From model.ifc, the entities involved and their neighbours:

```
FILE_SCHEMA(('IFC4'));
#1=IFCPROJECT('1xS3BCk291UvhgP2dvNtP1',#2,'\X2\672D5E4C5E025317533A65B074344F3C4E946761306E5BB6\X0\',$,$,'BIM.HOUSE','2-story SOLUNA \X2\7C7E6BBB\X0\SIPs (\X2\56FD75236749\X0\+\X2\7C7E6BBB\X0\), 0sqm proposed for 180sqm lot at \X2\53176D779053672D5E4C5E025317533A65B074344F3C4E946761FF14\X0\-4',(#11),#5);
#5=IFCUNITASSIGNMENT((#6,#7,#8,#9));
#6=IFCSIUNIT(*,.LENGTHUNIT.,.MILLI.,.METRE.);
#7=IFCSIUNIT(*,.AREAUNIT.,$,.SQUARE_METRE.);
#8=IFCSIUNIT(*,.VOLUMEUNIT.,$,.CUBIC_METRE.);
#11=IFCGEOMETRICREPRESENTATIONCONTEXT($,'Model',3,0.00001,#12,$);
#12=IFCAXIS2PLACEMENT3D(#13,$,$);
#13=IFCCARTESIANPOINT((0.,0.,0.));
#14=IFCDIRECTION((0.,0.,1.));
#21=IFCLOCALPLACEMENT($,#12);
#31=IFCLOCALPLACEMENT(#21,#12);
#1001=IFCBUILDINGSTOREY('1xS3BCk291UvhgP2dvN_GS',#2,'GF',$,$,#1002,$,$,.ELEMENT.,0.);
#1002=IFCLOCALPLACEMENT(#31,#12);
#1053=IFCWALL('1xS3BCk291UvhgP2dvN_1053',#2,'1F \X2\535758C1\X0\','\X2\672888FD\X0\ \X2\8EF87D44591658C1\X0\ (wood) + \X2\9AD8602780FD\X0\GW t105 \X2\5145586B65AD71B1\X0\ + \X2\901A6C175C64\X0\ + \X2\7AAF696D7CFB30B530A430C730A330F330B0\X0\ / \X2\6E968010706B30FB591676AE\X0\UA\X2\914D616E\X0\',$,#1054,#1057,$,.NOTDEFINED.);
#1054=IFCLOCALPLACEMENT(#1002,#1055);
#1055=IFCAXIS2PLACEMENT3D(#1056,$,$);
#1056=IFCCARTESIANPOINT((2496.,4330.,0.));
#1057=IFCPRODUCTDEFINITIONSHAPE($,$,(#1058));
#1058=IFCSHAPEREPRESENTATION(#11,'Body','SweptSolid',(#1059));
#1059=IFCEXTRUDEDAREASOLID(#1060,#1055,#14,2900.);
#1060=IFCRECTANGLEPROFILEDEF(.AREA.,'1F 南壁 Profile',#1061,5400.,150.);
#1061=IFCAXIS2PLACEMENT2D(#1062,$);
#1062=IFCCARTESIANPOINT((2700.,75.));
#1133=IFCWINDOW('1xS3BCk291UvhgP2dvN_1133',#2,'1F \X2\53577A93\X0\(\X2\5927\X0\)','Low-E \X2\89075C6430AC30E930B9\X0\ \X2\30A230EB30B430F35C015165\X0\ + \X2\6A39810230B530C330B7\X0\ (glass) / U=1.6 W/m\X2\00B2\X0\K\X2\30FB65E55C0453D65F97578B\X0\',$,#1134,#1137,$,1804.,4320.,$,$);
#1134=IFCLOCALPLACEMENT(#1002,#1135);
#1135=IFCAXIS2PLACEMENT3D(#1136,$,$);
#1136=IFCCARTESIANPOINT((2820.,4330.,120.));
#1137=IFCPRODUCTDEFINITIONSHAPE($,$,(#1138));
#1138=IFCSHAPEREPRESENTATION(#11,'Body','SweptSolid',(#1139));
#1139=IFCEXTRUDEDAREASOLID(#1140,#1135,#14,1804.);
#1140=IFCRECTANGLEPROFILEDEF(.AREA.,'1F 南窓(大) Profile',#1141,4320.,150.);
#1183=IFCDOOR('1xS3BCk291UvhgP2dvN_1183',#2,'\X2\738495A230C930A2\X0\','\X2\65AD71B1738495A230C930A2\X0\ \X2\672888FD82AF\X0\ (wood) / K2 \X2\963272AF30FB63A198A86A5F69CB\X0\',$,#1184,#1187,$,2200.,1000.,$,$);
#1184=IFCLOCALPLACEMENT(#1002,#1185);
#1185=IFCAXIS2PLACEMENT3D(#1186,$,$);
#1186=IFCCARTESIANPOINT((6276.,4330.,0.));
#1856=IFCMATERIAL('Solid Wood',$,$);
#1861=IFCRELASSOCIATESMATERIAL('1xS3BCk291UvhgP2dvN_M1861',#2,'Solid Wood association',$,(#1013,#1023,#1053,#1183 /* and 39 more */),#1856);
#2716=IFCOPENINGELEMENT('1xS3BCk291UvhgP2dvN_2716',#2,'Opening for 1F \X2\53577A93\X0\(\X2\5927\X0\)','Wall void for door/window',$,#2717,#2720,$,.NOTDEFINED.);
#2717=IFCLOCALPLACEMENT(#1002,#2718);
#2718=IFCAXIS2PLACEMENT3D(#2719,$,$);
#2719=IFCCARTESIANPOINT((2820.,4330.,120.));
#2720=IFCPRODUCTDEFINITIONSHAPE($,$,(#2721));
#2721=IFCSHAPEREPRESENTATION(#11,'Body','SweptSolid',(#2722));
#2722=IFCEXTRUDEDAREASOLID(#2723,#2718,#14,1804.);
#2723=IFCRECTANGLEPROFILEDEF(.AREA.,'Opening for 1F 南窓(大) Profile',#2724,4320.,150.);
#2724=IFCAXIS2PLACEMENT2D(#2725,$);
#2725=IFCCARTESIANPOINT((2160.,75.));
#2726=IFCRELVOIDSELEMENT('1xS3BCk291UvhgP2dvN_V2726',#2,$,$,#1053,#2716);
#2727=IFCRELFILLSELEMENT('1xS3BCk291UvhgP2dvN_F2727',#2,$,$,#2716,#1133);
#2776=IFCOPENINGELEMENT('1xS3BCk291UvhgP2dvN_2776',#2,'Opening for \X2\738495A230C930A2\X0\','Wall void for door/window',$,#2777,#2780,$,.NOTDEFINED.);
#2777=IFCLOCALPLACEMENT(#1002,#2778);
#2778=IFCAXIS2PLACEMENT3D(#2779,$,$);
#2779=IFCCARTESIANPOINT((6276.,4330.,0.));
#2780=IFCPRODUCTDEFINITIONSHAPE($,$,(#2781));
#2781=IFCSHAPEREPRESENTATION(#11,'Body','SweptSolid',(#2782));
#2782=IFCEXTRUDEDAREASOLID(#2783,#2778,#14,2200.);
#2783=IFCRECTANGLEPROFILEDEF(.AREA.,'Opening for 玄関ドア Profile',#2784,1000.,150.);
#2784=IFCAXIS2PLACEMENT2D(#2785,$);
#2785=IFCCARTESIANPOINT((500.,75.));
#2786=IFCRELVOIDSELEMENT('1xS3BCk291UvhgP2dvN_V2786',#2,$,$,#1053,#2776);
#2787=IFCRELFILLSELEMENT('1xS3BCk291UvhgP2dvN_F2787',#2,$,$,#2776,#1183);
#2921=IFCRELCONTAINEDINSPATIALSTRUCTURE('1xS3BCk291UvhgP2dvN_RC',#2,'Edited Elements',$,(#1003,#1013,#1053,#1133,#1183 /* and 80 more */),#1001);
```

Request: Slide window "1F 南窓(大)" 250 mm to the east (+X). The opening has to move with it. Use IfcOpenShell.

```python
import ifcopenshell
import ifcopenshell.api.geometry
import ifcopenshell.util.placement
import ifcopenshell.util.unit

model = ifcopenshell.open("model.ifc")
unit_scale = ifcopenshell.util.unit.calculate_unit_scale(model)

window = model.by_guid("1xS3BCk291UvhgP2dvN_1133")
opening = window.FillsVoids[0].RelatingOpeningElement
wall = opening.VoidsElements[0].RelatingBuildingElement

wall_matrix = ifcopenshell.util.placement.get_local_placement(wall.ObjectPlacement)
shift = wall_matrix[:3, 0] * 0.25 / unit_scale
before = ifcopenshell.util.placement.get_local_placement(window.ObjectPlacement)[:3, 3].copy()

# The window is not placed relative to its opening, so move both.
for product in (opening, window):
    matrix = ifcopenshell.util.placement.get_local_placement(product.ObjectPlacement)
    matrix[:3, 3] += shift
    ifcopenshell.api.geometry.edit_object_placement(model, product=product, matrix=matrix, is_si=False)

after = ifcopenshell.util.placement.get_local_placement(window.ObjectPlacement)[:3, 3]
print("window moved by", (after - before).round(3) + 0.0)

model.write("model_rev.ifc")
```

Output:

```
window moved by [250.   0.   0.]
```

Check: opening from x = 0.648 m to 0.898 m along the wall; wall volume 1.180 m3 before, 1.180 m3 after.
